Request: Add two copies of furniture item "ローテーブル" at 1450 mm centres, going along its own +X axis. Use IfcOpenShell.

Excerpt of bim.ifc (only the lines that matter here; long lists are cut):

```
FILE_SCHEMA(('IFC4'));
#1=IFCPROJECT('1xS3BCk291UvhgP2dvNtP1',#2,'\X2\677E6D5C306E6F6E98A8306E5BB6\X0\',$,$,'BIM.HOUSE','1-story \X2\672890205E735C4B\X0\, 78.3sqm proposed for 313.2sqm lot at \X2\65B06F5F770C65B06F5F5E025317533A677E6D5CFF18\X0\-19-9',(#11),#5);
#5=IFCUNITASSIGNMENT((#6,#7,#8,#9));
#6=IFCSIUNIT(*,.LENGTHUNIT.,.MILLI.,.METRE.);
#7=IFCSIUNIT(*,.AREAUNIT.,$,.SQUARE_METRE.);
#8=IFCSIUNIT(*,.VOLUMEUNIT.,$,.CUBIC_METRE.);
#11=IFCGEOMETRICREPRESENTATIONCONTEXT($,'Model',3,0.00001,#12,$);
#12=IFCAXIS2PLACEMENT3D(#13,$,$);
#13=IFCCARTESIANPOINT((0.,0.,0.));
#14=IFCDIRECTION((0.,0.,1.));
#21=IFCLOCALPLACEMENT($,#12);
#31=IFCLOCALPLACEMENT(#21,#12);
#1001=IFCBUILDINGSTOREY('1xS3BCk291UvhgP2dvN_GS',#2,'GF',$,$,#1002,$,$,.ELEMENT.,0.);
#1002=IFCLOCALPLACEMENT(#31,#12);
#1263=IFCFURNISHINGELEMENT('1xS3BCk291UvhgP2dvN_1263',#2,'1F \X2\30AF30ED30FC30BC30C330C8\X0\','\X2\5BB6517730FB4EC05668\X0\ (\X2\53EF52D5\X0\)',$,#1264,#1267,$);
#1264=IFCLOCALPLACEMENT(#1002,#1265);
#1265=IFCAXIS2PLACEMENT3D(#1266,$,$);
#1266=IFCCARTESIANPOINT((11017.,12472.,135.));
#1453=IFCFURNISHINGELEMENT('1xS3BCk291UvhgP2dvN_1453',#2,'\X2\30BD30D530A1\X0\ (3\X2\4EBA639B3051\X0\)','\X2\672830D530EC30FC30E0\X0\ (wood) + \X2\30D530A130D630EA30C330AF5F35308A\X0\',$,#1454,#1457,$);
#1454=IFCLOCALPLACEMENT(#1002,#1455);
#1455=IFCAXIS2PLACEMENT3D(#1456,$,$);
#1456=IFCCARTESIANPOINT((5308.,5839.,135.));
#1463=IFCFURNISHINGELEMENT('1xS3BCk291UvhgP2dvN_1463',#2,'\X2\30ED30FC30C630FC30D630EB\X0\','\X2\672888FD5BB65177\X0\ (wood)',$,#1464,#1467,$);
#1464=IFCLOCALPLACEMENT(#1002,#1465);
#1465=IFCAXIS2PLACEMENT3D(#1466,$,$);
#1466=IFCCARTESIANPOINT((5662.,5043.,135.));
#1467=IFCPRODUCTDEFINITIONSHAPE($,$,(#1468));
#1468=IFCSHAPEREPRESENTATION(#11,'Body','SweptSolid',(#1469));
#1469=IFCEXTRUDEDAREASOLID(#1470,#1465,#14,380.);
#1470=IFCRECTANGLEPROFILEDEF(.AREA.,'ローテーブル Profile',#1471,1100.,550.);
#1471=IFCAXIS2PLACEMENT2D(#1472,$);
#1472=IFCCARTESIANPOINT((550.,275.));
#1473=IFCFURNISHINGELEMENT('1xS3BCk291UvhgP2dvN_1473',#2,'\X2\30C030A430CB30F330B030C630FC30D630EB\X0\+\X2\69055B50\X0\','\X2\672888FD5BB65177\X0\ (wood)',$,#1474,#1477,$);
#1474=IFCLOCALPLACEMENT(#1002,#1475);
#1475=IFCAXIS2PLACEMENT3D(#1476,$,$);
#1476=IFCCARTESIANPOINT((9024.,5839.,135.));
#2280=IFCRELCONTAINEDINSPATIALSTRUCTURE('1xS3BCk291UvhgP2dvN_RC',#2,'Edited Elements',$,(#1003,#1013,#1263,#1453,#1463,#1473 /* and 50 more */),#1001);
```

```python
import ifcopenshell
import ifcopenshell.api.geometry
import ifcopenshell.api.root
import ifcopenshell.util.element
import ifcopenshell.util.placement
import ifcopenshell.util.unit

model = ifcopenshell.open("bim.ifc")
unit_scale = ifcopenshell.util.unit.calculate_unit_scale(model)


def reuse_history(source, copy):
    """copy_class also copies each property set's owner history, people and application; keep the originals."""
    for rel in copy.IsDefinedBy:
        if rel.is_a("IfcRelDefinesByProperties") and (history := rel.RelatingPropertyDefinition.OwnerHistory):
            rel.RelatingPropertyDefinition.OwnerHistory = source.OwnerHistory
            ifcopenshell.util.element.remove_deep2(model, history)


source = model.by_guid("1xS3BCk291UvhgP2dvN_1463")
base = ifcopenshell.util.placement.get_local_placement(source.ObjectPlacement)
step = base[:3, 0] * 1.45 / unit_scale

for i in range(1, 3):
    copy = ifcopenshell.api.root.copy_class(model, product=source)
    copy.Representation = ifcopenshell.util.element.copy_deep(
        model, source.Representation, exclude=["IfcGeometricRepresentationContext", "IfcRepresentationMap"]
    )
    reuse_history(source, copy)
    matrix = base.copy()
    matrix[:3, 3] += i * step
    print("added at", matrix[:3, 3].round(3) + 0.0)
    ifcopenshell.api.geometry.edit_object_placement(model, product=copy, matrix=matrix, is_si=False)

model.write("bim_updated.ifc")
```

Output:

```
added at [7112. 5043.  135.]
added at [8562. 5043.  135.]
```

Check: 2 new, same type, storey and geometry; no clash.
